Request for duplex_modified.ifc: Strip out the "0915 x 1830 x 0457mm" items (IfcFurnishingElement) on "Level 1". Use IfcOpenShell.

First a look at what the model holds.

```python
import ifcopenshell
import ifcopenshell.util.element

model = ifcopenshell.open("duplex_modified.ifc")
print(model.schema)
storey = next(s for s in model.by_type("IfcBuildingStorey") if s.Name == "Level 1")
furniture = [e for e in ifcopenshell.util.element.get_decomposition(storey) if e.is_a("IfcFurnishingElement")]
seen = {}
for e in furniture:
    element_type = ifcopenshell.util.element.get_type(e)
    name = element_type.Name if element_type not in (None, e) else None
    seen[name] = seen.get(name, 0) + 1
for name, count in sorted(seen.items(), key=str):
    print(count, "x", name)
```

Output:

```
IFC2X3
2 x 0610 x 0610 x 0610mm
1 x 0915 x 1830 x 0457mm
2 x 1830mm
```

```python
import ifcopenshell
import ifcopenshell.api.root
import ifcopenshell.util.element

model = ifcopenshell.open("duplex_modified.ifc")

storey = next(s for s in model.by_type("IfcBuildingStorey") if s.Name == "Level 1")
furniture = [e for e in ifcopenshell.util.element.get_decomposition(storey) if e.is_a("IfcFurnishingElement")]
targets = [e for e in furniture if (t := ifcopenshell.util.element.get_type(e)) not in (None, e) and t.Name == "0915 x 1830 x 0457mm"]

for e in targets:
    ifcopenshell.api.root.remove_product(model, product=e)
print(len(targets), "removed")

model.write("duplex_modified_updated.ifc")
```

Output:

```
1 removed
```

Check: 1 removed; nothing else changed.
